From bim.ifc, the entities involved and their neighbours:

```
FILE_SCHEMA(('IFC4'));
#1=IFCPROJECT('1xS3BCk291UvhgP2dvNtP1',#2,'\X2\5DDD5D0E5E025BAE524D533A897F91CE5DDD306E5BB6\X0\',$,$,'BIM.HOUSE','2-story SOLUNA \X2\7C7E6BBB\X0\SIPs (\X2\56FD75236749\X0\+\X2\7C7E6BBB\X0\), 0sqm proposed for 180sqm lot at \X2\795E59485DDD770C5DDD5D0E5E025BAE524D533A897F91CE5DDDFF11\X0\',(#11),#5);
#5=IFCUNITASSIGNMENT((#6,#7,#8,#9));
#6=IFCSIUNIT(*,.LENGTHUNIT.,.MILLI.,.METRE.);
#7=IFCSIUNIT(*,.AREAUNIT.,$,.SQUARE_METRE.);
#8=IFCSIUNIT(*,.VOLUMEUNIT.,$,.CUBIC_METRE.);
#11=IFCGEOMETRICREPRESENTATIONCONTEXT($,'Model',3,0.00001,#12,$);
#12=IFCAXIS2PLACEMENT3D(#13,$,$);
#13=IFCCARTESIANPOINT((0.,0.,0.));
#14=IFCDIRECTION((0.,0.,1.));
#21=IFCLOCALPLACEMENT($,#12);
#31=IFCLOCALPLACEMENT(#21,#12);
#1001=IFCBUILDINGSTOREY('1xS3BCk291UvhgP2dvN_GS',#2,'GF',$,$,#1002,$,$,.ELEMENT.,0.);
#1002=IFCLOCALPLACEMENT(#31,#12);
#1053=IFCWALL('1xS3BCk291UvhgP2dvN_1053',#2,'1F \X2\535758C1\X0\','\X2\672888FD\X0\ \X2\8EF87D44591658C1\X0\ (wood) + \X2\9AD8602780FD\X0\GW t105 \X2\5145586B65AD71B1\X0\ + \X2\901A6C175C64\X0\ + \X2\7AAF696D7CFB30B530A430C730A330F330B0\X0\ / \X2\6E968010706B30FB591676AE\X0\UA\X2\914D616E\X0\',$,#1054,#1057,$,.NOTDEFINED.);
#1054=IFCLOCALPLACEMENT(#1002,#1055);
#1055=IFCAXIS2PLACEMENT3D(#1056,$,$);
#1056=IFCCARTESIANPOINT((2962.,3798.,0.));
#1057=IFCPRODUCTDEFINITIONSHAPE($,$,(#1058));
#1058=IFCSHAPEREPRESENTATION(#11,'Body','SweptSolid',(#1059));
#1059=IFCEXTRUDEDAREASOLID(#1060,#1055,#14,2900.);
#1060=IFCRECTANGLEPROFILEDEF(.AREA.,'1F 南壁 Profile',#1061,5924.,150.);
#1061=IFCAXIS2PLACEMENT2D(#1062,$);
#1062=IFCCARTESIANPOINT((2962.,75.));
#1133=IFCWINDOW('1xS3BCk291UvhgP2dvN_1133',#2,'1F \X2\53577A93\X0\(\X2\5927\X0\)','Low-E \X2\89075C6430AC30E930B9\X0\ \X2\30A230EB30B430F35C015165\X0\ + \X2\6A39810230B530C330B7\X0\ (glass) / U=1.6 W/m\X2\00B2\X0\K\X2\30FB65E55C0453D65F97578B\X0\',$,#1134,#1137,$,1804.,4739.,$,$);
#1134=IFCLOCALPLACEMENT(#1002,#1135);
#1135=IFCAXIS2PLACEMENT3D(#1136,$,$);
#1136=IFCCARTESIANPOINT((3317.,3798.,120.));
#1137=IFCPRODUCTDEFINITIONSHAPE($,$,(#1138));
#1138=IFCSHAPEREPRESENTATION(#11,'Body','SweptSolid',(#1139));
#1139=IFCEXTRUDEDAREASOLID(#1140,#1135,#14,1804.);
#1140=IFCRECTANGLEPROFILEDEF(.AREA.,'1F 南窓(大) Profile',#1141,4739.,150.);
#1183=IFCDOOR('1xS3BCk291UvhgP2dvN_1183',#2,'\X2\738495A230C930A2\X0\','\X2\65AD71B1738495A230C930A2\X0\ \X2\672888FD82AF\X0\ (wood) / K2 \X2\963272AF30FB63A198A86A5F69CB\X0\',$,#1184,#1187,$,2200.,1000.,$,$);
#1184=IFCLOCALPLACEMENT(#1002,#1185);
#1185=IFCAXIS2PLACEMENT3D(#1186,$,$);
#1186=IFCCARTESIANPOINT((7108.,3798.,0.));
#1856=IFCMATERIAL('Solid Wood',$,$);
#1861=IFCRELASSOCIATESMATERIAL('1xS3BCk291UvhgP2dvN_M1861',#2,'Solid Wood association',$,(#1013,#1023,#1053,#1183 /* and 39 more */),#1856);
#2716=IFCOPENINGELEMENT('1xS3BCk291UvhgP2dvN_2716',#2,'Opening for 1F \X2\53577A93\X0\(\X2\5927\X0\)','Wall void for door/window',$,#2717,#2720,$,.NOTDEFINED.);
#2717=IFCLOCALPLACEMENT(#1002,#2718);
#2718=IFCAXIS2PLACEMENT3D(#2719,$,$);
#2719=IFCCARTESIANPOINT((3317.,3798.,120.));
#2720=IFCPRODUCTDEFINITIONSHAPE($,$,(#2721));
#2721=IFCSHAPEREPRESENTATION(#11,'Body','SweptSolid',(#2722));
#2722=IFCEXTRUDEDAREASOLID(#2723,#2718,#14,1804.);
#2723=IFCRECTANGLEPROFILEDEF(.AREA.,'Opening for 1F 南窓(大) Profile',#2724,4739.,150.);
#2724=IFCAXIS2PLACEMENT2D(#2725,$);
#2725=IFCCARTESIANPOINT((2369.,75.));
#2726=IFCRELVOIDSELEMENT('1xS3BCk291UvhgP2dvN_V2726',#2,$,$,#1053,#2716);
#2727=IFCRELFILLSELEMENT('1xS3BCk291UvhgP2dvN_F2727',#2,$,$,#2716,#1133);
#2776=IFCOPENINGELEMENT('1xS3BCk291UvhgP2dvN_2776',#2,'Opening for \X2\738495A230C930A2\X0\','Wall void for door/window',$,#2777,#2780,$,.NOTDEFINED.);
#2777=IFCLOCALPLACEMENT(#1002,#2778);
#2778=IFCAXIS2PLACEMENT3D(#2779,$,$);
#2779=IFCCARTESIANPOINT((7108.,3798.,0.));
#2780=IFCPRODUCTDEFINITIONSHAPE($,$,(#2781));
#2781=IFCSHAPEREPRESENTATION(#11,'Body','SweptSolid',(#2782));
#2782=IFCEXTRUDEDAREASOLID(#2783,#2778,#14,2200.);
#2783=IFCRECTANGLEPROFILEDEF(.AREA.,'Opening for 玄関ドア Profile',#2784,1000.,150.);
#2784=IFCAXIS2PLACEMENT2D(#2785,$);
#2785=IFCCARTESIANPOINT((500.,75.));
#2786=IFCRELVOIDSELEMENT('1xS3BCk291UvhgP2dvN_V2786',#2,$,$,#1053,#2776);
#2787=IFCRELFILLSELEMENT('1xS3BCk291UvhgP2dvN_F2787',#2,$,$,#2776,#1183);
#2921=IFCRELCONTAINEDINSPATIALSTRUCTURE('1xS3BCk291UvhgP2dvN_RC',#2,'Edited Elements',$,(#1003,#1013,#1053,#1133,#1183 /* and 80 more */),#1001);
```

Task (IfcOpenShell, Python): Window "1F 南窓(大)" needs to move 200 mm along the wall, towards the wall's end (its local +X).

```python
import ifcopenshell
import ifcopenshell.api.geometry
import ifcopenshell.util.placement

model = ifcopenshell.open("bim.ifc")

window = model.by_guid("1xS3BCk291UvhgP2dvN_1133")
opening = window.FillsVoids[0].RelatingOpeningElement
wall = opening.VoidsElements[0].RelatingBuildingElement

wall_matrix = ifcopenshell.util.placement.get_local_placement(wall.ObjectPlacement)
shift = wall_matrix[:3, 0] * 200.0
before = ifcopenshell.util.placement.get_local_placement(window.ObjectPlacement)[:3, 3].copy()

# The window is not placed relative to its opening, so move both.
for product in (opening, window):
    matrix = ifcopenshell.util.placement.get_local_placement(product.ObjectPlacement)
    matrix[:3, 3] += shift
    ifcopenshell.api.geometry.edit_object_placement(model, product=product, matrix=matrix, is_si=False)

after = ifcopenshell.util.placement.get_local_placement(window.ObjectPlacement)[:3, 3]
print("window moved by", (after - before).round(3) + 0.0)

model.write("bim_rev.ifc")
```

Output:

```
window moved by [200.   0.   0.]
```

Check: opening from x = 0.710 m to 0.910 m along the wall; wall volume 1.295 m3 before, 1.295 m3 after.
